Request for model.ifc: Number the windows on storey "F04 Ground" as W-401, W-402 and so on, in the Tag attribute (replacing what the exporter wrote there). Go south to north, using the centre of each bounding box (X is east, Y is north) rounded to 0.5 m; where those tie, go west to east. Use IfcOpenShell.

First a look at what the model holds.

```python
import ifcopenshell
import ifcopenshell.util.element
import ifcopenshell.util.placement

model = ifcopenshell.open("model.ifc")
print(model.schema)
storey = next(s for s in model.by_type("IfcBuildingStorey") if s.Name == "F04 Ground")
windows = [e for e in ifcopenshell.util.element.get_decomposition(storey) if e.is_a("IfcWindow")]
for e in sorted(windows, key=lambda e: e.id()):
    origin = ifcopenshell.util.placement.get_local_placement(e.ObjectPlacement)[:3, 3]
    print(e.id(), e.Tag, e.Name, origin.round(2) + 0.0, sep=" | ")
```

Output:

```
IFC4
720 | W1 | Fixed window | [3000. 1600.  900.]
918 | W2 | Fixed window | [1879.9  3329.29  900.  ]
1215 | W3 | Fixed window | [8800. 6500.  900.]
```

```python
import ifcopenshell
import ifcopenshell.geom
import ifcopenshell.util.element
import ifcopenshell.util.shape

model = ifcopenshell.open("model.ifc")
settings = ifcopenshell.geom.settings()
settings.set("use-world-coords", True)


def centre(element):
    shape = ifcopenshell.geom.create_shape(settings, element)
    return ifcopenshell.util.shape.get_bbox_centroid(shape.geometry)


storey = next(s for s in model.by_type("IfcBuildingStorey") if s.Name == "F04 Ground")
windows = [e for e in ifcopenshell.util.element.get_decomposition(storey) if e.is_a("IfcWindow")]

# Insertion points can sit at a corner or the storey origin, so sort by the geometry (in metres).
centres = {e: centre(e) for e in windows}
windows.sort(key=lambda e: (round(centres[e][1] / 0.5), centres[e][0]))

for i, e in enumerate(windows, start=1):
    number = f"W-4{i:02d}"
    e.Tag = number
    print(e.id(), number)

model.write("model_rev.ifc")
```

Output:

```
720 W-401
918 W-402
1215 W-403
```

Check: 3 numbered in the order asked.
